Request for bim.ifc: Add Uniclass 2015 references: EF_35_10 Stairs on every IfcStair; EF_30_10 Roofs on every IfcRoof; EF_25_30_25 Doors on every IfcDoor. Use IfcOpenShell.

First a look at what the model holds.

```python
import ifcopenshell

model = ifcopenshell.open("bim.ifc")
print(model.schema)
print("classifications:", [c.Name for c in model.by_type("IfcClassification")])
for ifc_class in ("IfcDoor", "IfcRoof", "IfcStair", "IfcWall", "IfcWindow"):
    print(ifc_class, len(model.by_type(ifc_class)))
```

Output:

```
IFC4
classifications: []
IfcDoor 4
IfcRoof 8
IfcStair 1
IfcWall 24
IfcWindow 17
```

```python
import ifcopenshell
import ifcopenshell.api.classification

model = ifcopenshell.open("bim.ifc")

system = ifcopenshell.api.classification.add_classification(model, classification="Uniclass 2015")

codes = {
    "IfcStair": ("EF_35_10", "Stairs"),
    "IfcRoof": ("EF_30_10", "Roofs"),
    "IfcDoor": ("EF_25_30_25", "Doors"),
}
for ifc_class, (code, name) in codes.items():
    products = model.by_type(ifc_class)
    ifcopenshell.api.classification.add_reference(
        model, products=products, classification=system, identification=code, name=name
    )
    print(code, len(products))

model.write("bim-out.ifc")
```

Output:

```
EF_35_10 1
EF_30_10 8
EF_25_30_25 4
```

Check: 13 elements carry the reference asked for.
